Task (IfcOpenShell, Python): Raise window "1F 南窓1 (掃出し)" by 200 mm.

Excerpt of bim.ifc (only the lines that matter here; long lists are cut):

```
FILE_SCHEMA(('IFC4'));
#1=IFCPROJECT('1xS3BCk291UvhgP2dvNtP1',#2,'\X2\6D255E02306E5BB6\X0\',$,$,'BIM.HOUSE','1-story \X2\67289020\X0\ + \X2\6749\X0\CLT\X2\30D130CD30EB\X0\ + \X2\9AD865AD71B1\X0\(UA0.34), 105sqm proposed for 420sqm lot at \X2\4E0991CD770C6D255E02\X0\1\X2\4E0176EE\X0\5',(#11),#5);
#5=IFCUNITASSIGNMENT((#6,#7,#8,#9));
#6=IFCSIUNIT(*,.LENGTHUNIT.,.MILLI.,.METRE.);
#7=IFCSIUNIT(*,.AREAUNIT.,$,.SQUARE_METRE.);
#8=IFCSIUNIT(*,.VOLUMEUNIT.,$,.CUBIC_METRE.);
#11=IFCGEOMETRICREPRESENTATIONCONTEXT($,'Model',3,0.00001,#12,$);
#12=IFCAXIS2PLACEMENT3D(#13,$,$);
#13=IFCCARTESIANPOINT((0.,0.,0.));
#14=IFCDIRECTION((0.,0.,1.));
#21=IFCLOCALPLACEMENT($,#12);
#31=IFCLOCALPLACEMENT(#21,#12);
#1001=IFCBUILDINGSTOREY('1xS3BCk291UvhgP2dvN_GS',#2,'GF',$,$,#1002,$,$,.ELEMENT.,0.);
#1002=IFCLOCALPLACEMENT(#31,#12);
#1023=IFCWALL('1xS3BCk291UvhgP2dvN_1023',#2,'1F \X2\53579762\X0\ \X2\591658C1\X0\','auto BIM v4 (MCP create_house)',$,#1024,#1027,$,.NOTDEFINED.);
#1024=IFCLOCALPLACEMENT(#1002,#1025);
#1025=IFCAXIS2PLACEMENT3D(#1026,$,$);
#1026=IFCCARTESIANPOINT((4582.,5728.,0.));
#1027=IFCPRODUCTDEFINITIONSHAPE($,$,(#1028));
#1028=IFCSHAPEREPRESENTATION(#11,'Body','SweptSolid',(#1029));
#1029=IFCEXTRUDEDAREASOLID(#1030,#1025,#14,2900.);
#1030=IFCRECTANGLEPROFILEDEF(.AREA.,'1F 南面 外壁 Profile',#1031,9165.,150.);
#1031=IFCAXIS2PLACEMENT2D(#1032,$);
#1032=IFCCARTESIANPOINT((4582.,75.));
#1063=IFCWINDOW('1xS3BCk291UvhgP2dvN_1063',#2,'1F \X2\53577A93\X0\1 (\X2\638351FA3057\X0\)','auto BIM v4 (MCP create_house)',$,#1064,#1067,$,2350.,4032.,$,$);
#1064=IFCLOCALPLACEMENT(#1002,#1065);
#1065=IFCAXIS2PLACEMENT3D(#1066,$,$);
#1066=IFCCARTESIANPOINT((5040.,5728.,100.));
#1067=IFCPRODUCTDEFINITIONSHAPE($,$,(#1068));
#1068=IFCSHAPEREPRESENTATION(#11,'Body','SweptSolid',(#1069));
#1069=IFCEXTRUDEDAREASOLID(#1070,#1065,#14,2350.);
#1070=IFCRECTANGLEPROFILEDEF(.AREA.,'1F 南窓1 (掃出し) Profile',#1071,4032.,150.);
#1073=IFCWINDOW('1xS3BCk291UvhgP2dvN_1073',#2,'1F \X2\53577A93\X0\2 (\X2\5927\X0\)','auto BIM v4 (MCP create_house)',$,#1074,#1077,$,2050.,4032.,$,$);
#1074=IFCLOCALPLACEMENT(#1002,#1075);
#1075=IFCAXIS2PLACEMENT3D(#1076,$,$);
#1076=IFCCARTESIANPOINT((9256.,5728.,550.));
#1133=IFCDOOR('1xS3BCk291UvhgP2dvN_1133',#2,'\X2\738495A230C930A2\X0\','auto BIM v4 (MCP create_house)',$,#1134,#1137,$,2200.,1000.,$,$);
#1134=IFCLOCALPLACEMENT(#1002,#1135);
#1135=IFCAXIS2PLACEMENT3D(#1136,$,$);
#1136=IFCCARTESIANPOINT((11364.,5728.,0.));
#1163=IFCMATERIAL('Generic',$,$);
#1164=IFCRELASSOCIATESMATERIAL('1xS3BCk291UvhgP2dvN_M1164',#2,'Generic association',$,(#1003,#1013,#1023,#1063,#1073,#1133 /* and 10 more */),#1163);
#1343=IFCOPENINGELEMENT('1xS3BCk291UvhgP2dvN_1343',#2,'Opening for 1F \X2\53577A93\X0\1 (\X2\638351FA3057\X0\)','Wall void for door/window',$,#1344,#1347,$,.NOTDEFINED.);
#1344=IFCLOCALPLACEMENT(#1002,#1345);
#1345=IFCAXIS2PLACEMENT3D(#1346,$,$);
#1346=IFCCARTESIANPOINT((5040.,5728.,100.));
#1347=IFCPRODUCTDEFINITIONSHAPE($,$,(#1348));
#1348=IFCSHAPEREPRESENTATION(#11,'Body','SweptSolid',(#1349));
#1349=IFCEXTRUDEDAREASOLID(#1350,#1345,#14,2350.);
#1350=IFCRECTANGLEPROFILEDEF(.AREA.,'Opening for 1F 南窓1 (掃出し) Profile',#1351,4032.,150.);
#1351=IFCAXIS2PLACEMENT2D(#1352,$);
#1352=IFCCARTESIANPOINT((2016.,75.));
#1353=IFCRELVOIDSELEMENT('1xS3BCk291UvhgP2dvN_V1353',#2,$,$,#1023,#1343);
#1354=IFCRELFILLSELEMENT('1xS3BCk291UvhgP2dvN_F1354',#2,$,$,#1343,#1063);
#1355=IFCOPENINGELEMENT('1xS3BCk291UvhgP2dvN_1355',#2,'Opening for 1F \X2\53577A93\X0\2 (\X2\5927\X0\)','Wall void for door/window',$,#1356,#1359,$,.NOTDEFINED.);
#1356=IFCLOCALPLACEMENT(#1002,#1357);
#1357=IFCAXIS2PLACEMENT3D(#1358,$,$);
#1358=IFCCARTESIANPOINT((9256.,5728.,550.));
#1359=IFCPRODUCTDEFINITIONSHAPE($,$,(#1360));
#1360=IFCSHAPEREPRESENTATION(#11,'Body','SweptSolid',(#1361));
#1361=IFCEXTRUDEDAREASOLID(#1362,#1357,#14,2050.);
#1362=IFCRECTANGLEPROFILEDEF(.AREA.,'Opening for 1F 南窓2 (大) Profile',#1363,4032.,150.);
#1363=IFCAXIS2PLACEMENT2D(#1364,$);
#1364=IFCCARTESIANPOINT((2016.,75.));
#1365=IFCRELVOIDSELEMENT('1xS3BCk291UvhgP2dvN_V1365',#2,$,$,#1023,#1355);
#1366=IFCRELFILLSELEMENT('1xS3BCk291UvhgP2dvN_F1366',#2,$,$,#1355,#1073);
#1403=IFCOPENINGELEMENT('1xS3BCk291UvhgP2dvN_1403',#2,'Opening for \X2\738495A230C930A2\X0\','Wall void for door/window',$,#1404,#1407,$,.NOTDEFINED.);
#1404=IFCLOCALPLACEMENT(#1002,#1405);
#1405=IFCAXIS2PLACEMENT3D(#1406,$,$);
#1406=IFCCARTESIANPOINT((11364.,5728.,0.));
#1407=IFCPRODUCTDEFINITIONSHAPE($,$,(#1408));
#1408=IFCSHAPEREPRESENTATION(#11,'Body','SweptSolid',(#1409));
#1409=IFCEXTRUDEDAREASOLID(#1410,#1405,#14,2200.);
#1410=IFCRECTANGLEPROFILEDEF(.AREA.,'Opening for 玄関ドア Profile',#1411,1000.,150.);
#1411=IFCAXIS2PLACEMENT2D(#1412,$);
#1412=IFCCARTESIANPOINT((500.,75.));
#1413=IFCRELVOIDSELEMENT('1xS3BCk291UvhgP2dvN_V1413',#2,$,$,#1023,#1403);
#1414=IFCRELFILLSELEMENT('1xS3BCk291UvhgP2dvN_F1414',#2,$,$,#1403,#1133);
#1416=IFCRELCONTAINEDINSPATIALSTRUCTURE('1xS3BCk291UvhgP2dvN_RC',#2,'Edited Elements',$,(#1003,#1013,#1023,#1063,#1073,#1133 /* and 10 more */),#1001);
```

```python
import numpy as np
import ifcopenshell
import ifcopenshell.api.geometry
import ifcopenshell.util.placement
import ifcopenshell.util.unit

model = ifcopenshell.open("bim.ifc")
unit_scale = ifcopenshell.util.unit.calculate_unit_scale(model)

window = model.by_guid("1xS3BCk291UvhgP2dvN_1063")
opening = window.FillsVoids[0].RelatingOpeningElement
dz = 0.2 / unit_scale

shift = np.array([0.0, 0.0, dz])
# The window is not placed relative to its opening, so move both.
for product in (opening, window):
    matrix = ifcopenshell.util.placement.get_local_placement(product.ObjectPlacement)
    matrix[:3, 3] += shift
    ifcopenshell.api.geometry.edit_object_placement(model, product=product, matrix=matrix, is_si=False)

print(f"moved by {dz * unit_scale:+.3f} m")

model.write("bim_updated.ifc")
```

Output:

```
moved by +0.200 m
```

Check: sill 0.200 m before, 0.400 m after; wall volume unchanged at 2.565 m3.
